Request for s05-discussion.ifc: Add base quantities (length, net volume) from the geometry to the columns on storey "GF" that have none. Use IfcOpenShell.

First a look at what the model holds.

```python
import ifcopenshell
import ifcopenshell.util.element
import ifcopenshell.util.unit

model = ifcopenshell.open("s05-discussion.ifc")
print(model.schema)
for unit_type in ("LENGTHUNIT", "AREAUNIT", "VOLUMEUNIT"):
    print(unit_type, ifcopenshell.util.unit.calculate_unit_scale(model, unit_type))
storey = next(s for s in model.by_type("IfcBuildingStorey") if s.Name == "GF")
columns = [e for e in ifcopenshell.util.element.get_decomposition(storey) if e.is_a("IfcColumn")]
for e in sorted(columns, key=lambda e: e.id()):
    print(e.id(), e.is_a(), e.Name, list(ifcopenshell.util.element.get_psets(e, qtos_only=True)), sep=" | ")
```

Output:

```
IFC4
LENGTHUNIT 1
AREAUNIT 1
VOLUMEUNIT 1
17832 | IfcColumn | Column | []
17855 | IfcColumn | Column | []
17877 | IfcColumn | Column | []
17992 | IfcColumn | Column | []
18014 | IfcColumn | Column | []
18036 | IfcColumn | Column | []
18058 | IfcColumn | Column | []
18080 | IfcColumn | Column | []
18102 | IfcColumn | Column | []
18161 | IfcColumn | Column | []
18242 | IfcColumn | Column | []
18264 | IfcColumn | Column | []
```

```python
import ifcopenshell
import ifcopenshell.api.pset
import ifcopenshell.geom
import ifcopenshell.util.element
import ifcopenshell.util.shape
import ifcopenshell.util.unit

model = ifcopenshell.open("s05-discussion.ifc")
unit_scale = ifcopenshell.util.unit.calculate_unit_scale(model)
volume_scale = ifcopenshell.util.unit.calculate_unit_scale(model, "VOLUMEUNIT")
settings = ifcopenshell.geom.settings()

storey = next(s for s in model.by_type("IfcBuildingStorey") if s.Name == "GF")
columns = [e for e in ifcopenshell.util.element.get_decomposition(storey) if e.is_a("IfcColumn")]

for e in sorted(columns, key=lambda e: e.id()):
    if ifcopenshell.util.element.get_psets(e, qtos_only=True, should_inherit=False):
        continue
    # Geometry comes back in metres, in the element's own axes.
    shape = ifcopenshell.geom.create_shape(settings, e)
    values = {
        "Length": ifcopenshell.util.shape.get_z(shape.geometry) / unit_scale,
        "NetVolume": ifcopenshell.util.shape.get_volume(shape.geometry) / volume_scale,
    }
    qto = ifcopenshell.api.pset.add_qto(model, product=e, name="Qto_ColumnBaseQuantities")
    ifcopenshell.api.pset.edit_qto(model, qto=qto, properties=values)
    print(e.id(), {k: round(v, 3) for k, v in values.items()})

model.write("s05-discussion_updated.ifc")
```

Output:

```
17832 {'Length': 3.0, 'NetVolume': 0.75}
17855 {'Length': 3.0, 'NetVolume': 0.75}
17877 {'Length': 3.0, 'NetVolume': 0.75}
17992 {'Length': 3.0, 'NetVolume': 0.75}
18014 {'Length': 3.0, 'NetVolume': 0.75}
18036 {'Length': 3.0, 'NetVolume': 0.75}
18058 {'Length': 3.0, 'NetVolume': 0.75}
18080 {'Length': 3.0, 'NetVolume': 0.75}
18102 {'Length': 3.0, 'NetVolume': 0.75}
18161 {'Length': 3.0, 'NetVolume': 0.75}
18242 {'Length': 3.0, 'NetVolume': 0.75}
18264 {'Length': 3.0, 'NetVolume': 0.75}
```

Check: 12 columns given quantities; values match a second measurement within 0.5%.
